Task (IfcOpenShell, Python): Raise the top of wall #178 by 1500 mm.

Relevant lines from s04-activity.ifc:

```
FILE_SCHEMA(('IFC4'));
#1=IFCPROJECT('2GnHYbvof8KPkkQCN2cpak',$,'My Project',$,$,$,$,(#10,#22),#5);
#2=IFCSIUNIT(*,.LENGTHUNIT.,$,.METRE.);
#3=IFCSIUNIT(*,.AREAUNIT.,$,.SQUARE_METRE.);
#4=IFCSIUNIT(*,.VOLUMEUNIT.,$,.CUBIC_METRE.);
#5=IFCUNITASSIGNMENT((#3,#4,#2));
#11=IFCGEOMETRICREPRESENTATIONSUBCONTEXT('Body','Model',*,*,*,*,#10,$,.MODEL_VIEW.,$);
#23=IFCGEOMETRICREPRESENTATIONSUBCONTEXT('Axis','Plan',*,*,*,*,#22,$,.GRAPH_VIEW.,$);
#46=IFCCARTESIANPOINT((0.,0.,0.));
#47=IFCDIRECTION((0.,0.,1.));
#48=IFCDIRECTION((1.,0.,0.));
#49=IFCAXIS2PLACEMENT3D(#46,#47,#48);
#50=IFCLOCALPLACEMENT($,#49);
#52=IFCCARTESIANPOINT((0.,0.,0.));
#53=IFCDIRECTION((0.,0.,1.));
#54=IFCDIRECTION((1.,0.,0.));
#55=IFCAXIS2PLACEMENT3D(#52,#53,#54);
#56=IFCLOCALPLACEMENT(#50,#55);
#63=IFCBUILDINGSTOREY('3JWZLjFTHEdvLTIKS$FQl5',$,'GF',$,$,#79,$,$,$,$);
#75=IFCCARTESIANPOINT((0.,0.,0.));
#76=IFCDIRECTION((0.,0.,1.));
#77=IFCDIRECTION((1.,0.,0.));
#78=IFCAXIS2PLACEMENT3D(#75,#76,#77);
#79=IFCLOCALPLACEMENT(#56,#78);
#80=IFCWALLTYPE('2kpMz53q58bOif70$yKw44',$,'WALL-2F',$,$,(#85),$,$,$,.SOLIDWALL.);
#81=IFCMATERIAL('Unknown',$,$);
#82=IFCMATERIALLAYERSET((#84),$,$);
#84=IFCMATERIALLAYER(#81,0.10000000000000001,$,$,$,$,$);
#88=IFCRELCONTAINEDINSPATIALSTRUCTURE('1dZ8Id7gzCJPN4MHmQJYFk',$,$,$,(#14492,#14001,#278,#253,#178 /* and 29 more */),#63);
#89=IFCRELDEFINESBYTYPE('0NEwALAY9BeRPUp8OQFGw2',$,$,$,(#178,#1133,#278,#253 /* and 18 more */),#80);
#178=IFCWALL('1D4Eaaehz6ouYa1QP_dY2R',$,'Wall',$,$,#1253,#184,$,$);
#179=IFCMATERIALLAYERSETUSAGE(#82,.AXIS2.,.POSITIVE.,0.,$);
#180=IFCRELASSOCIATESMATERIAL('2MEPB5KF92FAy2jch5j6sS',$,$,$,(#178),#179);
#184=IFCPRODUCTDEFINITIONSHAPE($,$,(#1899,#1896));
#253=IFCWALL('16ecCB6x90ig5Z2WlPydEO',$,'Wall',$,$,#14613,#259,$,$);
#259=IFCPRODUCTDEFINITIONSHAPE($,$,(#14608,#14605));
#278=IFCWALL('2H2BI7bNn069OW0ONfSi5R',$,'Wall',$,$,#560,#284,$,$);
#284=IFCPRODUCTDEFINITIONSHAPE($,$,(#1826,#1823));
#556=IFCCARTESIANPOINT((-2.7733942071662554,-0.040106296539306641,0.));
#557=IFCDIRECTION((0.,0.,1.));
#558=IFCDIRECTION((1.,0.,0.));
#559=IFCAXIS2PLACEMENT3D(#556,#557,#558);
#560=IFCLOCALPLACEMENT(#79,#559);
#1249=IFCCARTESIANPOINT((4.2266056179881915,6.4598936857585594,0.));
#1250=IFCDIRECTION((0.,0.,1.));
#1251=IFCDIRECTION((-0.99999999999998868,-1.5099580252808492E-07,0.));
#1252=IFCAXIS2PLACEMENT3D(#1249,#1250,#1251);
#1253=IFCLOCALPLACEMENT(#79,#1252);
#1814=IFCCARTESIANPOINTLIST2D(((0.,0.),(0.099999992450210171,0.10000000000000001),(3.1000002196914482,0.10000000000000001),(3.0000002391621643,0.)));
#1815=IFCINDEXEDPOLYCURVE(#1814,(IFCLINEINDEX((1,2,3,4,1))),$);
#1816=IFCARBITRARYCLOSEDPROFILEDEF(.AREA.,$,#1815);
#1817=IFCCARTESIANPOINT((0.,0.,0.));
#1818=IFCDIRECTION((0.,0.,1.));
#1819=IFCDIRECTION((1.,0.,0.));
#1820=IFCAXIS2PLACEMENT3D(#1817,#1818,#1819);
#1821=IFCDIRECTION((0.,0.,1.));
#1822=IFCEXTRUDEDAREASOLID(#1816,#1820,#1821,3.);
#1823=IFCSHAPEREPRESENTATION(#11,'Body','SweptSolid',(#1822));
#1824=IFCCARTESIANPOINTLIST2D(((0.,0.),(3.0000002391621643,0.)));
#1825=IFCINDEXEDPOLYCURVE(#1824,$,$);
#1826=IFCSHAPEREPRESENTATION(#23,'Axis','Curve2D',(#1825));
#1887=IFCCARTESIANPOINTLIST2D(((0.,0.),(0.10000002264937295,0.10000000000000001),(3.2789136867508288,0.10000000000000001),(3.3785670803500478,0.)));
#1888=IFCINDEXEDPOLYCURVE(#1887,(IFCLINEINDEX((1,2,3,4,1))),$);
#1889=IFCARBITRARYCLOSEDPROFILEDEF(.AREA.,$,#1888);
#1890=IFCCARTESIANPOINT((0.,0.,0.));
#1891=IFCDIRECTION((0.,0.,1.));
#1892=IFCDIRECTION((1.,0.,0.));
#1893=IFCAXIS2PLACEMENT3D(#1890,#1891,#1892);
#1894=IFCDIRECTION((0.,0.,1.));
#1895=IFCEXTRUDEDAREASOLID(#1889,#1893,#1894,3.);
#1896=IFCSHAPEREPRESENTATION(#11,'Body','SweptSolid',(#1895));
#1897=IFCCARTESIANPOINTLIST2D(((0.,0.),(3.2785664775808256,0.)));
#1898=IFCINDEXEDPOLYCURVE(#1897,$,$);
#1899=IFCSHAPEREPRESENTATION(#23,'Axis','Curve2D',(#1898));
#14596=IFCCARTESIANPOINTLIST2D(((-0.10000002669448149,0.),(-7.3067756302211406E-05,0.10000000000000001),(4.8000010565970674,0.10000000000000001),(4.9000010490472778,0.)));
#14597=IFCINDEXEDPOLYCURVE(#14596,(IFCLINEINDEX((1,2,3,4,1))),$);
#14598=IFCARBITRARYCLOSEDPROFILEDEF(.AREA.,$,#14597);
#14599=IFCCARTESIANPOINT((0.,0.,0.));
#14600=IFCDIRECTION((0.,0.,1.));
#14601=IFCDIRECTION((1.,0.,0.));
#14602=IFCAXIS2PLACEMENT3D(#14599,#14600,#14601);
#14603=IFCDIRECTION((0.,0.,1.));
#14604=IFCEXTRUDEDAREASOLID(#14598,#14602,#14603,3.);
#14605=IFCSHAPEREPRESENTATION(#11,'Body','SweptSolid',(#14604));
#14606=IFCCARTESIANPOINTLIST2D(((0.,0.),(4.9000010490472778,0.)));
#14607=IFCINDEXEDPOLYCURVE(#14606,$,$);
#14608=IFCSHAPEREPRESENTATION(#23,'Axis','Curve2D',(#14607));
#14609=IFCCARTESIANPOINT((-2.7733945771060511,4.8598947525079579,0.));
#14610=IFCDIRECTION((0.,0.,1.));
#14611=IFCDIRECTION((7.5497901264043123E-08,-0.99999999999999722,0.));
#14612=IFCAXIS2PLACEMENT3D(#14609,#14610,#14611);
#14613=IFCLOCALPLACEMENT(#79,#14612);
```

```python
import ifcopenshell
import ifcopenshell.geom
import ifcopenshell.util.representation
import ifcopenshell.util.shape

model = ifcopenshell.open("s04-activity.ifc")
settings = ifcopenshell.geom.settings()


def volume(element):
    """Net volume in cubic metres, openings subtracted."""
    shape = ifcopenshell.geom.create_shape(settings, element)
    return ifcopenshell.util.shape.get_volume(shape.geometry)


wall = model.by_guid("1D4Eaaehz6ouYa1QP_dY2R")
before = volume(wall)

body = ifcopenshell.util.representation.get_representation(wall, "Model", "Body")
solid = body.Items[0]
old_height = solid.Depth
solid.Depth += 1.5
after = volume(wall)

print(f"height {old_height:g} -> {solid.Depth:g}, volume {before:.3f} -> {after:.3f} m3")

model.write("s04-activity-out.ifc")
```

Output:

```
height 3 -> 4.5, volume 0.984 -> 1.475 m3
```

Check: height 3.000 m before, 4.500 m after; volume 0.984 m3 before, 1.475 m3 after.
